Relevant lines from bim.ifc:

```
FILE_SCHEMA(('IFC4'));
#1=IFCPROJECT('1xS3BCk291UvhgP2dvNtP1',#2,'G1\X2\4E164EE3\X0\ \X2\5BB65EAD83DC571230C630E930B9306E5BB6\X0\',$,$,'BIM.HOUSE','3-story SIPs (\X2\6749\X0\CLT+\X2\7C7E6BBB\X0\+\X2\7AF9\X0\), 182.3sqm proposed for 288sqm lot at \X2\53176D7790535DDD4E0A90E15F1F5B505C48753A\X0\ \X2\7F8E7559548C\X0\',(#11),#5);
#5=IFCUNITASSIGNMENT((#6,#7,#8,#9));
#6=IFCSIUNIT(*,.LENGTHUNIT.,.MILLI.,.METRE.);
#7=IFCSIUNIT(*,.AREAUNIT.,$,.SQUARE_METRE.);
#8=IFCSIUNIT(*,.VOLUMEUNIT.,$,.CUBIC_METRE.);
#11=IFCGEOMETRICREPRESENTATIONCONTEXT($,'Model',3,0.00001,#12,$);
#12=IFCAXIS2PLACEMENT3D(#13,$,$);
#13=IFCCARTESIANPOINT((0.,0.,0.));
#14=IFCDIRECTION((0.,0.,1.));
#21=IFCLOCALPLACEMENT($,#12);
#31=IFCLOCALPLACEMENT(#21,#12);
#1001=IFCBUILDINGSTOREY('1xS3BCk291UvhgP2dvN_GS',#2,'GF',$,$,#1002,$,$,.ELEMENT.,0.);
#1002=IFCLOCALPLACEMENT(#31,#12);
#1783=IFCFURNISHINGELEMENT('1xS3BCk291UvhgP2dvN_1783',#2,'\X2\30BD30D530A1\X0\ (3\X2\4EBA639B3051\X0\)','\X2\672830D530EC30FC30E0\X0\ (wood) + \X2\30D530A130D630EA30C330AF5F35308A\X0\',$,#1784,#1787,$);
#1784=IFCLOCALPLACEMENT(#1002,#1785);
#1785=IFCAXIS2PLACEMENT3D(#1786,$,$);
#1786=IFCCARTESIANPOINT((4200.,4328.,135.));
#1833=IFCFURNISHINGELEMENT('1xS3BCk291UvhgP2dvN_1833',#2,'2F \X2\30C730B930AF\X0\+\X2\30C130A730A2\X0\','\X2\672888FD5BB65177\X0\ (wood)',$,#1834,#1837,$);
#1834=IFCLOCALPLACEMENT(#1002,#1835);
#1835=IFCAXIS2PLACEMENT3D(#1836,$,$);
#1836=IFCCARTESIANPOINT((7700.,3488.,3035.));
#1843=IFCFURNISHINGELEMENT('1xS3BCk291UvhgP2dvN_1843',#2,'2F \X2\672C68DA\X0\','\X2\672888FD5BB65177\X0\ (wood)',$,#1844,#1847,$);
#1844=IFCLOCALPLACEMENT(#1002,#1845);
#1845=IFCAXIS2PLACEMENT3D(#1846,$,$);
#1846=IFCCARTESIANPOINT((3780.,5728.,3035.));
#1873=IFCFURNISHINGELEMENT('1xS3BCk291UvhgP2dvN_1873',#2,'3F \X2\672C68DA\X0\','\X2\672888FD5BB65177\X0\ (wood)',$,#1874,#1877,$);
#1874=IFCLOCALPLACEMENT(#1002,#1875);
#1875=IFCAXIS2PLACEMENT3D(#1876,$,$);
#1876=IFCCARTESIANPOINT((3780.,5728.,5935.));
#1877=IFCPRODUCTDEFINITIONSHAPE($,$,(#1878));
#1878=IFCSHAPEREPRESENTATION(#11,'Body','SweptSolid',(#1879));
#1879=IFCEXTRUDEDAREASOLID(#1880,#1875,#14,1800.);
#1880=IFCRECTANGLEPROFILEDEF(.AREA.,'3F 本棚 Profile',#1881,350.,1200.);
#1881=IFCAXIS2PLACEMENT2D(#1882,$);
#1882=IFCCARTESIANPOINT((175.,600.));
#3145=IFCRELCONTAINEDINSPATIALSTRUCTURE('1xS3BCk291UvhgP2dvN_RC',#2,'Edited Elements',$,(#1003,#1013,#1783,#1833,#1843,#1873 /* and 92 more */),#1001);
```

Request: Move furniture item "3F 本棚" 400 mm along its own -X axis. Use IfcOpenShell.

```python
import ifcopenshell
import ifcopenshell.api.geometry
import ifcopenshell.util.placement
import ifcopenshell.util.unit

model = ifcopenshell.open("bim.ifc")
unit_scale = ifcopenshell.util.unit.calculate_unit_scale(model)

item = model.by_guid("1xS3BCk291UvhgP2dvN_1873")
matrix = ifcopenshell.util.placement.get_local_placement(item.ObjectPlacement)
matrix[:3, 3] -= matrix[:3, 0] * 0.4 / unit_scale
ifcopenshell.api.geometry.edit_object_placement(model, product=item, matrix=matrix, is_si=False)

print(ifcopenshell.util.placement.get_local_placement(item.ObjectPlacement).round(3) + 0.0)

model.write("bim_rev.ifc")
```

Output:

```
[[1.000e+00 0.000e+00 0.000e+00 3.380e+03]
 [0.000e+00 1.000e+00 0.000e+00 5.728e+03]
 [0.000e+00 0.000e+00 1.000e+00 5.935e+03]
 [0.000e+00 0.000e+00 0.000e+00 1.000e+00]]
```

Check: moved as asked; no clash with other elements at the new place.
